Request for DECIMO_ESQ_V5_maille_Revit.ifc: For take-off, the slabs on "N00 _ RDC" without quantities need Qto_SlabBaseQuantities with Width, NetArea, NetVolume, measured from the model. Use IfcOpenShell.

First a look at what the model holds.

```python
import ifcopenshell
import ifcopenshell.util.element
import ifcopenshell.util.unit

model = ifcopenshell.open("DECIMO_ESQ_V5_maille_Revit.ifc")
print(model.schema)
for unit_type in ("LENGTHUNIT", "AREAUNIT", "VOLUMEUNIT"):
    print(unit_type, ifcopenshell.util.unit.calculate_unit_scale(model, unit_type))
storey = next(s for s in model.by_type("IfcBuildingStorey") if s.Name == "N00 _ RDC")
slabs = [e for e in ifcopenshell.util.element.get_decomposition(storey) if e.is_a("IfcSlab")]
for e in sorted(slabs, key=lambda e: e.id()):
    print(e.id(), e.is_a(), e.Name, list(ifcopenshell.util.element.get_psets(e, qtos_only=True)), sep=" | ")
```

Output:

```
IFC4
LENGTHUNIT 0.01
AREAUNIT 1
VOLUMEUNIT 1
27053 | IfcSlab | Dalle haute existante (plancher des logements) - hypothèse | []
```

```python
import ifcopenshell
import ifcopenshell.api.pset
import ifcopenshell.geom
import ifcopenshell.util.element
import ifcopenshell.util.shape
import ifcopenshell.util.unit

model = ifcopenshell.open("DECIMO_ESQ_V5_maille_Revit.ifc")
unit_scale = ifcopenshell.util.unit.calculate_unit_scale(model)
area_scale = ifcopenshell.util.unit.calculate_unit_scale(model, "AREAUNIT")
volume_scale = ifcopenshell.util.unit.calculate_unit_scale(model, "VOLUMEUNIT")
settings = ifcopenshell.geom.settings()

storey = next(s for s in model.by_type("IfcBuildingStorey") if s.Name == "N00 _ RDC")
slabs = [e for e in ifcopenshell.util.element.get_decomposition(storey) if e.is_a("IfcSlab")]

for e in sorted(slabs, key=lambda e: e.id()):
    if ifcopenshell.util.element.get_psets(e, qtos_only=True, should_inherit=False):
        continue
    # Geometry comes back in metres, in the element's own axes.
    shape = ifcopenshell.geom.create_shape(settings, e)
    values = {
        "Width": ifcopenshell.util.shape.get_z(shape.geometry) / unit_scale,
        "NetArea": ifcopenshell.util.shape.get_footprint_area(shape.geometry) / area_scale,
        "NetVolume": ifcopenshell.util.shape.get_volume(shape.geometry) / volume_scale,
    }
    qto = ifcopenshell.api.pset.add_qto(model, product=e, name="Qto_SlabBaseQuantities")
    ifcopenshell.api.pset.edit_qto(model, qto=qto, properties=values)
    print(e.id(), {k: round(v, 3) for k, v in values.items()})

model.write("DECIMO_ESQ_V5_maille_Revit_v2.ifc")
```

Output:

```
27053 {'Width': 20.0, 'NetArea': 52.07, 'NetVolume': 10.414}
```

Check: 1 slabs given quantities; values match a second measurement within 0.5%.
